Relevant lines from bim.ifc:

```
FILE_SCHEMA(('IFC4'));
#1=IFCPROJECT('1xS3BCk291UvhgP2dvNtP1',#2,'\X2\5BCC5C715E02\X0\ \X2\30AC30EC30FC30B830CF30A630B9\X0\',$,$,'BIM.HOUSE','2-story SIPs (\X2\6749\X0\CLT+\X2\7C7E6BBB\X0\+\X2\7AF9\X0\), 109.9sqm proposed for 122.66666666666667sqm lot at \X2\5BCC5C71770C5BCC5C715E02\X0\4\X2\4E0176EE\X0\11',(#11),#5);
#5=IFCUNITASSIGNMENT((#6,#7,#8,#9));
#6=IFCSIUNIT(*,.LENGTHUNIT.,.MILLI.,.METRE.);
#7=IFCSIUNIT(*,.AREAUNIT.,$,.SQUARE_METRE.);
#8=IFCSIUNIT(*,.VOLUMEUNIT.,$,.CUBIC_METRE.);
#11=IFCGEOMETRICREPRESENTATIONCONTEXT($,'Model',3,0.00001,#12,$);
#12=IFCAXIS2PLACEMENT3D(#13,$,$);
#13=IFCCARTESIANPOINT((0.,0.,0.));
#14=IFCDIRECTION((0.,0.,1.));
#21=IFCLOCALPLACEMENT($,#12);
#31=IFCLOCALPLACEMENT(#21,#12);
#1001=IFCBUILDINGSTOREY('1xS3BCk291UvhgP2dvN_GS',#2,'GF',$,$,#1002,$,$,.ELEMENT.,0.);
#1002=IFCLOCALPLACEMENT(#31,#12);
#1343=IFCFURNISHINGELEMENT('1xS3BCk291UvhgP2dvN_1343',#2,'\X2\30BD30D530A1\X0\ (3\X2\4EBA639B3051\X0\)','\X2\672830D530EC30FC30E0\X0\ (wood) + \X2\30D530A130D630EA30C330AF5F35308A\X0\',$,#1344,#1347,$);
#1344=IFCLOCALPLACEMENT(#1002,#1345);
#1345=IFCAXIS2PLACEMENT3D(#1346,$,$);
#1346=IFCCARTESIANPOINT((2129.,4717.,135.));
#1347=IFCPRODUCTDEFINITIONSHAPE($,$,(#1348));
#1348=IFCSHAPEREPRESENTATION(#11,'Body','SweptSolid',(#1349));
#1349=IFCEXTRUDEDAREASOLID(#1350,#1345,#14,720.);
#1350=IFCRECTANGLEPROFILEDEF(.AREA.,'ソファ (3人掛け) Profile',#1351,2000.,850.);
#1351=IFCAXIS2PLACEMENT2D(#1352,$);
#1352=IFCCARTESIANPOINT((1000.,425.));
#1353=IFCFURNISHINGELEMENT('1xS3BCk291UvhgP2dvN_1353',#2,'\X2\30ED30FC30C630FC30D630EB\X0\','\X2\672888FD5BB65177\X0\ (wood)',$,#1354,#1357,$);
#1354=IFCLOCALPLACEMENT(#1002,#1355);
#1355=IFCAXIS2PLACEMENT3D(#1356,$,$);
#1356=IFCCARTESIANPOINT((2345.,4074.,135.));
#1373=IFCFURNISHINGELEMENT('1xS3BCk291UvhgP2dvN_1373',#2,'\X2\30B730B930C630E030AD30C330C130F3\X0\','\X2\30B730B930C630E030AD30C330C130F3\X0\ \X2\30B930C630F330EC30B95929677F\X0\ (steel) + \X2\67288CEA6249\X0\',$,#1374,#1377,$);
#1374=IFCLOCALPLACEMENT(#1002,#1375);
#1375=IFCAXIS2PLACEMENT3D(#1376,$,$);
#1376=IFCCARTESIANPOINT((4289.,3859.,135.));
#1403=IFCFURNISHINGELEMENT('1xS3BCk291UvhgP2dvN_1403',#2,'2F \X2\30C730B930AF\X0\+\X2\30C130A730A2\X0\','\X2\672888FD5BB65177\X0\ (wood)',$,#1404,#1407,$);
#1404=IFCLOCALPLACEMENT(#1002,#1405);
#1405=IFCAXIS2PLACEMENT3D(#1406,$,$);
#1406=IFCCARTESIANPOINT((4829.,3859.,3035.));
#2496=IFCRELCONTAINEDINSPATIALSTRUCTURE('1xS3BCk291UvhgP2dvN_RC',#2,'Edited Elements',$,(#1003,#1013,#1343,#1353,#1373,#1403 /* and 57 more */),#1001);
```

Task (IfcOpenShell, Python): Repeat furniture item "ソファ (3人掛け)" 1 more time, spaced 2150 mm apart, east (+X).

```python
import numpy as np
import ifcopenshell
import ifcopenshell.api.geometry
import ifcopenshell.api.root
import ifcopenshell.util.element
import ifcopenshell.util.placement
import ifcopenshell.util.unit

model = ifcopenshell.open("bim.ifc")
unit_scale = ifcopenshell.util.unit.calculate_unit_scale(model)


def reuse_history(source, copy):
    """copy_class also copies each property set's owner history, people and application; keep the originals."""
    for rel in copy.IsDefinedBy:
        if rel.is_a("IfcRelDefinesByProperties") and (history := rel.RelatingPropertyDefinition.OwnerHistory):
            rel.RelatingPropertyDefinition.OwnerHistory = source.OwnerHistory
            ifcopenshell.util.element.remove_deep2(model, history)


source = model.by_guid("1xS3BCk291UvhgP2dvN_1343")
base = ifcopenshell.util.placement.get_local_placement(source.ObjectPlacement)
step = np.array([1.0, 0.0, 0.0]) * 2.15 / unit_scale

for i in range(1, 2):
    copy = ifcopenshell.api.root.copy_class(model, product=source)
    copy.Representation = ifcopenshell.util.element.copy_deep(
        model, source.Representation, exclude=["IfcGeometricRepresentationContext", "IfcRepresentationMap"]
    )
    reuse_history(source, copy)
    matrix = base.copy()
    matrix[:3, 3] += i * step
    print("added at", matrix[:3, 3].round(3) + 0.0)
    ifcopenshell.api.geometry.edit_object_placement(model, product=copy, matrix=matrix, is_si=False)

model.write("bim_rev.ifc")
```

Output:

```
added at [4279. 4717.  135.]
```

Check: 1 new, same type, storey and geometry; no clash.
